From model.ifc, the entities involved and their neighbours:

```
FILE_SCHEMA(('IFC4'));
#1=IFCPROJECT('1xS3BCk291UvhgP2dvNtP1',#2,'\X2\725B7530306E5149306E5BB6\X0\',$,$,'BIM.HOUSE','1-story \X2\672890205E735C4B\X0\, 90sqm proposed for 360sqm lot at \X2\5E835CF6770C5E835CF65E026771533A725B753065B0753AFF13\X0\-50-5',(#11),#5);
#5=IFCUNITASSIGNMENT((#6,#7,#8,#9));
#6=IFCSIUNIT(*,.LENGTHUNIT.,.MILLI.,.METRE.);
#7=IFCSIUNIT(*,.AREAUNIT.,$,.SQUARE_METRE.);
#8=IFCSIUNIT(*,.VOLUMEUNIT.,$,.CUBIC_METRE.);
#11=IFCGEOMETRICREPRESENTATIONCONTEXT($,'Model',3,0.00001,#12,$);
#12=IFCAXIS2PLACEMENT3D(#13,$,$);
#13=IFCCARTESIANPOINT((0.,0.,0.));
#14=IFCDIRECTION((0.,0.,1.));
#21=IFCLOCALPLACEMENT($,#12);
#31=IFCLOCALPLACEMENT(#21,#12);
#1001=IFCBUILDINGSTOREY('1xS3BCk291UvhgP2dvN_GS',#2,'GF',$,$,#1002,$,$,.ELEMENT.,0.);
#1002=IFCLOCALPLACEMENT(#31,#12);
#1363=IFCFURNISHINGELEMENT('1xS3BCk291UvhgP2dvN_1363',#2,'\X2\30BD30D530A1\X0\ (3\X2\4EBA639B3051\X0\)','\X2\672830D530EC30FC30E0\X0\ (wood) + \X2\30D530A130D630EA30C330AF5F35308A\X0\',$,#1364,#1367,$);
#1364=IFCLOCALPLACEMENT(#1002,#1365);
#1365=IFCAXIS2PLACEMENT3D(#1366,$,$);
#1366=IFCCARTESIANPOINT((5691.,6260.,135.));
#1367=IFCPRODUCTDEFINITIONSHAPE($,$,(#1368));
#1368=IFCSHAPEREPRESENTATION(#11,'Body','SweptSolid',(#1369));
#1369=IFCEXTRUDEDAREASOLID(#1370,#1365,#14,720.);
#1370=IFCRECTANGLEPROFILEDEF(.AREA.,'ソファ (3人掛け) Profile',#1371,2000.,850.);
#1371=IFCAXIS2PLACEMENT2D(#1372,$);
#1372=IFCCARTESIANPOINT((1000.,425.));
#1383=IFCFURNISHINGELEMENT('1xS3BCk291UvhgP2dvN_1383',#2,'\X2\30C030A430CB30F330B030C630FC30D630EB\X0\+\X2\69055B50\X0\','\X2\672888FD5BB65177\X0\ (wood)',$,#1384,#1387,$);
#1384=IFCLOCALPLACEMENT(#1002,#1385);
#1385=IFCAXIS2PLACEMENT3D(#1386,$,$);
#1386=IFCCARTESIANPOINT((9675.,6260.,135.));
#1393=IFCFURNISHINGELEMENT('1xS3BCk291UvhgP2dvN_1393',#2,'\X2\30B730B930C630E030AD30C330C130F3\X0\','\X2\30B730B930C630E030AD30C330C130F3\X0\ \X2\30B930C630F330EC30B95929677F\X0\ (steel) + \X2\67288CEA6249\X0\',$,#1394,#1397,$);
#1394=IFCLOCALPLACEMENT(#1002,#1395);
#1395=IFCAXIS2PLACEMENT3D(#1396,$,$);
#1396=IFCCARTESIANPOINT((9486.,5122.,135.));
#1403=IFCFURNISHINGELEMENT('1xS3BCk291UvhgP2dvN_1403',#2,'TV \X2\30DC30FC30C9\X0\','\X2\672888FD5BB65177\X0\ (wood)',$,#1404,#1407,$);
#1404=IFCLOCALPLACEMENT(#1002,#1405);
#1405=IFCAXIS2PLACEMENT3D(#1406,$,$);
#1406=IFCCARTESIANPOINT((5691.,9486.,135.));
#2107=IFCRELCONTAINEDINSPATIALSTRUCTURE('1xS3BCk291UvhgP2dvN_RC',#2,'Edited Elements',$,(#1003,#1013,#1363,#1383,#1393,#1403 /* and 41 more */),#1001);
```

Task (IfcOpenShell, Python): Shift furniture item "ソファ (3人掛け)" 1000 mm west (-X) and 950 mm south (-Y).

```python
import ifcopenshell
import ifcopenshell.api.geometry
import ifcopenshell.util.placement

model = ifcopenshell.open("model.ifc")

item = model.by_id(1363)
matrix = ifcopenshell.util.placement.get_local_placement(item.ObjectPlacement)
matrix[0, 3] -= 1000.0
matrix[1, 3] -= 950.0
ifcopenshell.api.geometry.edit_object_placement(model, product=item, matrix=matrix, is_si=False)

print(ifcopenshell.util.placement.get_local_placement(item.ObjectPlacement).round(3) + 0.0)

model.write("model_v2.ifc")
```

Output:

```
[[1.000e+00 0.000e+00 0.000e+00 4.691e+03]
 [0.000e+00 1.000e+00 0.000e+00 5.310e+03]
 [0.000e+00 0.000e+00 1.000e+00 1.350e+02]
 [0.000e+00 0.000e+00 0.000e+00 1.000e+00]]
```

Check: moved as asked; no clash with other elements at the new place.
